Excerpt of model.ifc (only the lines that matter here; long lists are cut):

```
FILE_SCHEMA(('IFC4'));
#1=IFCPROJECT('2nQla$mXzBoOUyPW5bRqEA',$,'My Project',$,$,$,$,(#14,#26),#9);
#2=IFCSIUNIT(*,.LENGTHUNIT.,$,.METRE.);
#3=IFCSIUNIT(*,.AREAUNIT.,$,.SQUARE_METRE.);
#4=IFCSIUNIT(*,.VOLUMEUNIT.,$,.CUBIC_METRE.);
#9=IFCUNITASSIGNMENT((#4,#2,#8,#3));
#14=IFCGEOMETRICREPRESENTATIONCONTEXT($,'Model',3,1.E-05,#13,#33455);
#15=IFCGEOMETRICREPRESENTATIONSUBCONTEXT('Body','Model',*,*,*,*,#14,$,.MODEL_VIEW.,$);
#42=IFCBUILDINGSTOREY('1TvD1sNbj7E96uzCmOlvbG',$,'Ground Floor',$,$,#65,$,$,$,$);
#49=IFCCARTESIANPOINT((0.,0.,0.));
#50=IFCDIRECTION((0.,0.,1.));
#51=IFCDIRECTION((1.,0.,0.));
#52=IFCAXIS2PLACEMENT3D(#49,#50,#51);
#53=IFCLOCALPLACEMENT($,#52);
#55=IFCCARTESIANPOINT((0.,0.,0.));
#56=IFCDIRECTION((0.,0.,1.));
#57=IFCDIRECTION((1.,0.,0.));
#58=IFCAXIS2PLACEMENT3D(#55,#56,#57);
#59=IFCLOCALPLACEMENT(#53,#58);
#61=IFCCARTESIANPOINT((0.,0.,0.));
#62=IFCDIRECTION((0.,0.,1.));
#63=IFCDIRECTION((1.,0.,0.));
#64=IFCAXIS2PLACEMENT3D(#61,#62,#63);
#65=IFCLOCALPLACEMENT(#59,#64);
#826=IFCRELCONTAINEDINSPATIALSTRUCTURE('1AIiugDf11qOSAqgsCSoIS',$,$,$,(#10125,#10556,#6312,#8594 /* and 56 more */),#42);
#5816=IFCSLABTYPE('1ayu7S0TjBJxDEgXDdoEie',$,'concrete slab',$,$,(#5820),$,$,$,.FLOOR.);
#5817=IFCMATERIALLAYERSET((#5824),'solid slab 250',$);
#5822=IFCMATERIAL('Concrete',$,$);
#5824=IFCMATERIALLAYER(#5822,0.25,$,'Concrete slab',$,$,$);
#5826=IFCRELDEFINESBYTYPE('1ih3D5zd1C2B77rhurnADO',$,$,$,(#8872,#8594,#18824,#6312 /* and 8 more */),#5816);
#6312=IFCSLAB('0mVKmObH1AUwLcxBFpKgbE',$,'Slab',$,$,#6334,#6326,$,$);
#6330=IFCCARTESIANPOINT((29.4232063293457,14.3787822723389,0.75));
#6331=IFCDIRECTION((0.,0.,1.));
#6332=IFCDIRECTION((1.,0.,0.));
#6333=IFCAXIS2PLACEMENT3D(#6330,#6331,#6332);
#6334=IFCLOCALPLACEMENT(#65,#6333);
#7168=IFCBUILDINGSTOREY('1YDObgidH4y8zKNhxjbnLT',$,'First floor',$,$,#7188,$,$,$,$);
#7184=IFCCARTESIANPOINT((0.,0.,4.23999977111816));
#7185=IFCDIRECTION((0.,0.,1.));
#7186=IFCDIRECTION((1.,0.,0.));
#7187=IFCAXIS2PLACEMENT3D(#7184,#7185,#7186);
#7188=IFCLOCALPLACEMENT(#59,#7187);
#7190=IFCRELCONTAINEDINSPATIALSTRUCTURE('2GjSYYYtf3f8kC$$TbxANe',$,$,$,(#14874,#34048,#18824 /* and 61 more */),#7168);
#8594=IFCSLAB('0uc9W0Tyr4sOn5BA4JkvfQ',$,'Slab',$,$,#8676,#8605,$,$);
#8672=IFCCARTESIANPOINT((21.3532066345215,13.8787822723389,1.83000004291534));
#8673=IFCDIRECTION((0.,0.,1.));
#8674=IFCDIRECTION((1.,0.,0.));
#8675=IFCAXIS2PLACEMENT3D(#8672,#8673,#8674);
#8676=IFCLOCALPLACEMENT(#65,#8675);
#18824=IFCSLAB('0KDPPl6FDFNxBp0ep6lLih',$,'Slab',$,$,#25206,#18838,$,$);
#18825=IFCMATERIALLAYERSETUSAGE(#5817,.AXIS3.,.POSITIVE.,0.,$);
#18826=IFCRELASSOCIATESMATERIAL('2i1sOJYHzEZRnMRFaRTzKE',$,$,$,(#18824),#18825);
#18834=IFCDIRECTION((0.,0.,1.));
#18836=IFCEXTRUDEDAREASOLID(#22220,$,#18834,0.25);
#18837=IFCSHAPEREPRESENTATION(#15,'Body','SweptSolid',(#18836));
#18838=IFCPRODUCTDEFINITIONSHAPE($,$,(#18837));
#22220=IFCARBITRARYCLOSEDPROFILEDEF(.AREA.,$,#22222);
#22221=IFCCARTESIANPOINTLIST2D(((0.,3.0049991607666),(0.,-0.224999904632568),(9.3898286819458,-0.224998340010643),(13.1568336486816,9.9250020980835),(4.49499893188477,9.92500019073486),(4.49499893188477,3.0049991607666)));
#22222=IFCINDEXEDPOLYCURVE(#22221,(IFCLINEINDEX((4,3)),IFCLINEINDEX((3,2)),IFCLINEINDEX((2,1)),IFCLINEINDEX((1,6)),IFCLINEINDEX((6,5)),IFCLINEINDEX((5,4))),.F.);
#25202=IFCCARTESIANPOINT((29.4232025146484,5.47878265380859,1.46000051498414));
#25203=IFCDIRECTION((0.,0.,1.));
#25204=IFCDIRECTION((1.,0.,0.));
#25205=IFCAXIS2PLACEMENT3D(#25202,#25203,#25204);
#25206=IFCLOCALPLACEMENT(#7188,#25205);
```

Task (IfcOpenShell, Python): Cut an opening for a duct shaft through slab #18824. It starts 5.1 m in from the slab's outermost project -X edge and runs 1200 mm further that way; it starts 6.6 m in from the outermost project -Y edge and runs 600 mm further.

```python
import numpy as np
import ifcopenshell
import ifcopenshell.api.feature
import ifcopenshell.api.geometry
import ifcopenshell.api.root
import ifcopenshell.geom
import ifcopenshell.util.placement
import ifcopenshell.util.representation
import ifcopenshell.util.shape
import ifcopenshell.util.unit

model = ifcopenshell.open("model.ifc")
unit_scale = ifcopenshell.util.unit.calculate_unit_scale(model)
settings = ifcopenshell.geom.settings()


def volume(element):
    """Net volume in cubic metres, openings subtracted."""
    shape = ifcopenshell.geom.create_shape(settings, element)
    return ifcopenshell.util.shape.get_volume(shape.geometry)


slab = model.by_id(18824)
before = volume(slab)

# Extent in the slab's own axes, in metres. The edges named are its -X and -Y sides.
slab_shape = ifcopenshell.geom.create_shape(settings, slab)
vertices = ifcopenshell.util.shape.get_vertices(slab_shape.geometry)
x_min, y_min, bottom = vertices.min(axis=0)
top = vertices[:, 2].max()

opening = ifcopenshell.api.root.create_entity(model, ifc_class="IfcOpeningElement", name="Duct shaft opening", predefined_type="OPENING")
context = ifcopenshell.util.representation.get_context(model, "Model", "Body", "MODEL_VIEW")
width, depth = 1.2, 0.6
outline = [(0.0, 0.0), (width, 0.0), (width, depth), (0.0, depth), (0.0, 0.0)]
# Overshoot both faces by 50 mm so the cut is clean.
shape = ifcopenshell.api.geometry.add_slab_representation(
    model, context=context, depth=top - bottom + 0.1, polyline=outline
)
ifcopenshell.api.geometry.assign_representation(model, product=opening, representation=shape)

matrix = ifcopenshell.util.placement.get_local_placement(slab.ObjectPlacement)
matrix[:, 3] = matrix @ np.append(np.array([x_min + 5.1, y_min + 6.6, bottom - 0.05]) / unit_scale, 1.0)
ifcopenshell.api.geometry.edit_object_placement(model, product=opening, matrix=matrix, is_si=False)
ifcopenshell.api.feature.add_feature(model, feature=opening, element=slab)

after = volume(slab)

print(f"slab volume {before:.3f} -> {after:.3f} m3")

model.write("model_v2.ifc")
```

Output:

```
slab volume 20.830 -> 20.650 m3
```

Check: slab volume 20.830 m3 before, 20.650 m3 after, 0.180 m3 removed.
